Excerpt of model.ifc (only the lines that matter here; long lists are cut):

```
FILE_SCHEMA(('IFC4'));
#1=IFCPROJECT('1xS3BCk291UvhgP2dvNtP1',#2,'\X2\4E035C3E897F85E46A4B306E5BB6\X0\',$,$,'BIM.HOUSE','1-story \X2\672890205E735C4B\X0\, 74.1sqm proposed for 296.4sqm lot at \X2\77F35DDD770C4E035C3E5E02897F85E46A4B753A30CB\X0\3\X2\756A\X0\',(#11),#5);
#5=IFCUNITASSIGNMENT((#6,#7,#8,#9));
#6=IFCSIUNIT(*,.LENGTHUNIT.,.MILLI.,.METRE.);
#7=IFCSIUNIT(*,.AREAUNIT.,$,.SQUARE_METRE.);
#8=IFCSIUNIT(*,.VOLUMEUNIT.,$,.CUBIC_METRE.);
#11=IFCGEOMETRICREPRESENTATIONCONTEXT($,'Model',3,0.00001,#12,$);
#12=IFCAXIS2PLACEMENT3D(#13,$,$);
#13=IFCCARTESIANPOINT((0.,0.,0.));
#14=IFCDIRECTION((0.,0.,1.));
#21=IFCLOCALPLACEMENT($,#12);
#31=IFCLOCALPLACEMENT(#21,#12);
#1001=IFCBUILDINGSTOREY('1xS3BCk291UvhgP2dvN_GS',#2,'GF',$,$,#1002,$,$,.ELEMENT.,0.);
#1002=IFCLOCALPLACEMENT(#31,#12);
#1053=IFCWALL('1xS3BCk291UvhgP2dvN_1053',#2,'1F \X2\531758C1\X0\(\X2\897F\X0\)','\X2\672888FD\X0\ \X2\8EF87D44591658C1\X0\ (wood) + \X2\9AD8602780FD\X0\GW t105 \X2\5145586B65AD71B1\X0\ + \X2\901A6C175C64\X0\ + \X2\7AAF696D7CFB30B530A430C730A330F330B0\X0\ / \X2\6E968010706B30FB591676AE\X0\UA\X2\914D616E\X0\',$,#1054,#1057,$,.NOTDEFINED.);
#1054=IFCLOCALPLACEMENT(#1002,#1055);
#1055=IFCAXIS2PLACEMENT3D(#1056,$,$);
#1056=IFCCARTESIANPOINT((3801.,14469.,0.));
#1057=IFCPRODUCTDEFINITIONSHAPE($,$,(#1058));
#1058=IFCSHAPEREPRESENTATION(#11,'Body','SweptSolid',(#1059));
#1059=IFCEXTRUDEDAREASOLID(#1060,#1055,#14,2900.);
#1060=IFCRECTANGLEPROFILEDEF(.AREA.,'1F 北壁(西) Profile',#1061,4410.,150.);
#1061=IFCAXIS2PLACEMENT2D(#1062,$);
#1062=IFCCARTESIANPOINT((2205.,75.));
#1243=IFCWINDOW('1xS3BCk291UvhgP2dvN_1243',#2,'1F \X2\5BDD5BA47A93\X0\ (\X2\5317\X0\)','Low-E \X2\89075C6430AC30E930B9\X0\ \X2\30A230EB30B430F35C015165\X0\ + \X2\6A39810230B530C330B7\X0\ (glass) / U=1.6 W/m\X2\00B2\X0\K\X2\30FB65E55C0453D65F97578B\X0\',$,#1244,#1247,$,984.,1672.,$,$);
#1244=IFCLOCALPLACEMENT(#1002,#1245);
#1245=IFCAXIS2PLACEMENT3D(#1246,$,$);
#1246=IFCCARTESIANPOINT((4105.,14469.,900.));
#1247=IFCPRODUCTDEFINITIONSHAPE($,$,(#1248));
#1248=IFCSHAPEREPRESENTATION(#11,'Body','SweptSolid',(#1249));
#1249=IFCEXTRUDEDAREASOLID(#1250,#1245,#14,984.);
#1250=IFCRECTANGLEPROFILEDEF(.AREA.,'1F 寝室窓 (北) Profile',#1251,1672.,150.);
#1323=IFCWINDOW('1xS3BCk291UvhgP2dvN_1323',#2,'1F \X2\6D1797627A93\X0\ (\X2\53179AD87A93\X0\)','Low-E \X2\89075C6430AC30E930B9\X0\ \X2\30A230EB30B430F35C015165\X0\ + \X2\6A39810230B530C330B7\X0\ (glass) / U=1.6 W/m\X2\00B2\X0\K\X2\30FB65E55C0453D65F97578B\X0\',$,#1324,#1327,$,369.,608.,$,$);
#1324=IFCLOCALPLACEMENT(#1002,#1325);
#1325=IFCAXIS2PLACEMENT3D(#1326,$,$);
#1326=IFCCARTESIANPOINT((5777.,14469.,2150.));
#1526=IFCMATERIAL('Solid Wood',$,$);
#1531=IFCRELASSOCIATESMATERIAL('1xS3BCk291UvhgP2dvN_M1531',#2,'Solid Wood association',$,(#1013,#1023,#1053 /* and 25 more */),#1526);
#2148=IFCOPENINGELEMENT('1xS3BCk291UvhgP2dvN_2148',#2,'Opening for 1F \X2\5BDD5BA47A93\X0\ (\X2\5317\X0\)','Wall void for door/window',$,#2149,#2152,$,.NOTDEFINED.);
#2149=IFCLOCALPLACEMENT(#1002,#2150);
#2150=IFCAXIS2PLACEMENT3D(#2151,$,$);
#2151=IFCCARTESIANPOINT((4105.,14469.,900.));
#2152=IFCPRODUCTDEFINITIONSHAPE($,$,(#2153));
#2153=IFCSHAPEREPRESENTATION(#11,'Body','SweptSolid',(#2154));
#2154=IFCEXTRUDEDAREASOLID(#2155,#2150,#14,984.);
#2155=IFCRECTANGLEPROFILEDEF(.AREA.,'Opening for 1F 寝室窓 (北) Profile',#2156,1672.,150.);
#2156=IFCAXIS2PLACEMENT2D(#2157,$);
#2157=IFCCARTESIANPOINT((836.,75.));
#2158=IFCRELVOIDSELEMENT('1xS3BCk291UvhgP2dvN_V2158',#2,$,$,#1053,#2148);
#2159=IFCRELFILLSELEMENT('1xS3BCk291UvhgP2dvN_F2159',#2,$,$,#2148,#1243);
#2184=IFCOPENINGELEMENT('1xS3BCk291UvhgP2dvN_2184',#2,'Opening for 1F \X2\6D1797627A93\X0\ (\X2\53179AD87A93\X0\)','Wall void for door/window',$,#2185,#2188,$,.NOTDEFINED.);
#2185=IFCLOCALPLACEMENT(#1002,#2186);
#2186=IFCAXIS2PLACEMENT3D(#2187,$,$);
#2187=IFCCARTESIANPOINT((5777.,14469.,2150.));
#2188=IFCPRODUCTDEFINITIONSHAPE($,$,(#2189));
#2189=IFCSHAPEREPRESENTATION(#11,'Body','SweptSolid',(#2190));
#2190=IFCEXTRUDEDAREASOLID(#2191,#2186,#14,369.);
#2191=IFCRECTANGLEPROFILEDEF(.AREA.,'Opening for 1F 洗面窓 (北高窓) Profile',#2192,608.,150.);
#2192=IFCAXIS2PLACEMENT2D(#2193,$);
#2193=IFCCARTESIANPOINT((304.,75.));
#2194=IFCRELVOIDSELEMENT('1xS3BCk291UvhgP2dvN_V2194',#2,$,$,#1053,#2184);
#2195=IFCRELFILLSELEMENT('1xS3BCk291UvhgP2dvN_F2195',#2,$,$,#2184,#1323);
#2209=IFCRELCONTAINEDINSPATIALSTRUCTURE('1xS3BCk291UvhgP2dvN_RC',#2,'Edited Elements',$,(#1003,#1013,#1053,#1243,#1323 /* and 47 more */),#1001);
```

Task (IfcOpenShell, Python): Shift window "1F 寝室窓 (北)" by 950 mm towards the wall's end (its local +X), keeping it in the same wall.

```python
import ifcopenshell
import ifcopenshell.api.geometry
import ifcopenshell.util.placement

model = ifcopenshell.open("model.ifc")

window = model.by_guid("1xS3BCk291UvhgP2dvN_1243")
opening = window.FillsVoids[0].RelatingOpeningElement
wall = opening.VoidsElements[0].RelatingBuildingElement

wall_matrix = ifcopenshell.util.placement.get_local_placement(wall.ObjectPlacement)
shift = wall_matrix[:3, 0] * 950.0
before = ifcopenshell.util.placement.get_local_placement(window.ObjectPlacement)[:3, 3].copy()

# The window is not placed relative to its opening, so move both.
for product in (opening, window):
    matrix = ifcopenshell.util.placement.get_local_placement(product.ObjectPlacement)
    matrix[:3, 3] += shift
    ifcopenshell.api.geometry.edit_object_placement(model, product=product, matrix=matrix, is_si=False)

after = ifcopenshell.util.placement.get_local_placement(window.ObjectPlacement)[:3, 3]
print("window moved by", (after - before).round(3) + 0.0)

model.write("model_edited.ifc")
```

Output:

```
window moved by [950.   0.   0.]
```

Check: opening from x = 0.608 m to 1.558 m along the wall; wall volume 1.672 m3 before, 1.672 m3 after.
